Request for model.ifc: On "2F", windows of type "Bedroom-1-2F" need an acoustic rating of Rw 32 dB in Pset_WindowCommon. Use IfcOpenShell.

First a look at what the model holds.

```python
import ifcopenshell
import ifcopenshell.util.element

model = ifcopenshell.open("model.ifc")
print(model.schema)
storey = next(s for s in model.by_type("IfcBuildingStorey") if s.Name == "2F")
windows = [e for e in ifcopenshell.util.element.get_decomposition(storey) if e.is_a("IfcWindow")]
seen = {}
for e in windows:
    element_type = ifcopenshell.util.element.get_type(e)
    key = (element_type.Name if element_type != e and element_type else None, ifcopenshell.util.element.get_pset(e, "Pset_WindowCommon", "AcousticRating"))
    seen[key] = seen.get(key, 0) + 1
for (name, value), count in sorted(seen.items(), key=str):
    print(count, "x", name, "|", value)
```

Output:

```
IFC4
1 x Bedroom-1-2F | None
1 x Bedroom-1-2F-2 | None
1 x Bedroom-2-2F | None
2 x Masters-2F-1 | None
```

```python
import ifcopenshell
import ifcopenshell.api.pset
import ifcopenshell.util.element

model = ifcopenshell.open("model.ifc")

storey = next(s for s in model.by_type("IfcBuildingStorey") if s.Name == "2F")
windows = [e for e in ifcopenshell.util.element.get_decomposition(storey) if e.is_a("IfcWindow")]

count = 0
for e in windows:
    element_type = ifcopenshell.util.element.get_type(e)
    if element_type in (None, e) or element_type.Name != "Bedroom-1-2F":
        continue
    # add_pset returns the element's existing set when there is one.
    pset = ifcopenshell.api.pset.add_pset(model, product=e, name="Pset_WindowCommon")
    ifcopenshell.api.pset.edit_pset(model, pset=pset, properties={"AcousticRating": "Rw 32 dB"})
    count += 1

print(count, "windows updated")

model.write("model_v2.ifc")
```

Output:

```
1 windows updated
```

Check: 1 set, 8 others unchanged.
